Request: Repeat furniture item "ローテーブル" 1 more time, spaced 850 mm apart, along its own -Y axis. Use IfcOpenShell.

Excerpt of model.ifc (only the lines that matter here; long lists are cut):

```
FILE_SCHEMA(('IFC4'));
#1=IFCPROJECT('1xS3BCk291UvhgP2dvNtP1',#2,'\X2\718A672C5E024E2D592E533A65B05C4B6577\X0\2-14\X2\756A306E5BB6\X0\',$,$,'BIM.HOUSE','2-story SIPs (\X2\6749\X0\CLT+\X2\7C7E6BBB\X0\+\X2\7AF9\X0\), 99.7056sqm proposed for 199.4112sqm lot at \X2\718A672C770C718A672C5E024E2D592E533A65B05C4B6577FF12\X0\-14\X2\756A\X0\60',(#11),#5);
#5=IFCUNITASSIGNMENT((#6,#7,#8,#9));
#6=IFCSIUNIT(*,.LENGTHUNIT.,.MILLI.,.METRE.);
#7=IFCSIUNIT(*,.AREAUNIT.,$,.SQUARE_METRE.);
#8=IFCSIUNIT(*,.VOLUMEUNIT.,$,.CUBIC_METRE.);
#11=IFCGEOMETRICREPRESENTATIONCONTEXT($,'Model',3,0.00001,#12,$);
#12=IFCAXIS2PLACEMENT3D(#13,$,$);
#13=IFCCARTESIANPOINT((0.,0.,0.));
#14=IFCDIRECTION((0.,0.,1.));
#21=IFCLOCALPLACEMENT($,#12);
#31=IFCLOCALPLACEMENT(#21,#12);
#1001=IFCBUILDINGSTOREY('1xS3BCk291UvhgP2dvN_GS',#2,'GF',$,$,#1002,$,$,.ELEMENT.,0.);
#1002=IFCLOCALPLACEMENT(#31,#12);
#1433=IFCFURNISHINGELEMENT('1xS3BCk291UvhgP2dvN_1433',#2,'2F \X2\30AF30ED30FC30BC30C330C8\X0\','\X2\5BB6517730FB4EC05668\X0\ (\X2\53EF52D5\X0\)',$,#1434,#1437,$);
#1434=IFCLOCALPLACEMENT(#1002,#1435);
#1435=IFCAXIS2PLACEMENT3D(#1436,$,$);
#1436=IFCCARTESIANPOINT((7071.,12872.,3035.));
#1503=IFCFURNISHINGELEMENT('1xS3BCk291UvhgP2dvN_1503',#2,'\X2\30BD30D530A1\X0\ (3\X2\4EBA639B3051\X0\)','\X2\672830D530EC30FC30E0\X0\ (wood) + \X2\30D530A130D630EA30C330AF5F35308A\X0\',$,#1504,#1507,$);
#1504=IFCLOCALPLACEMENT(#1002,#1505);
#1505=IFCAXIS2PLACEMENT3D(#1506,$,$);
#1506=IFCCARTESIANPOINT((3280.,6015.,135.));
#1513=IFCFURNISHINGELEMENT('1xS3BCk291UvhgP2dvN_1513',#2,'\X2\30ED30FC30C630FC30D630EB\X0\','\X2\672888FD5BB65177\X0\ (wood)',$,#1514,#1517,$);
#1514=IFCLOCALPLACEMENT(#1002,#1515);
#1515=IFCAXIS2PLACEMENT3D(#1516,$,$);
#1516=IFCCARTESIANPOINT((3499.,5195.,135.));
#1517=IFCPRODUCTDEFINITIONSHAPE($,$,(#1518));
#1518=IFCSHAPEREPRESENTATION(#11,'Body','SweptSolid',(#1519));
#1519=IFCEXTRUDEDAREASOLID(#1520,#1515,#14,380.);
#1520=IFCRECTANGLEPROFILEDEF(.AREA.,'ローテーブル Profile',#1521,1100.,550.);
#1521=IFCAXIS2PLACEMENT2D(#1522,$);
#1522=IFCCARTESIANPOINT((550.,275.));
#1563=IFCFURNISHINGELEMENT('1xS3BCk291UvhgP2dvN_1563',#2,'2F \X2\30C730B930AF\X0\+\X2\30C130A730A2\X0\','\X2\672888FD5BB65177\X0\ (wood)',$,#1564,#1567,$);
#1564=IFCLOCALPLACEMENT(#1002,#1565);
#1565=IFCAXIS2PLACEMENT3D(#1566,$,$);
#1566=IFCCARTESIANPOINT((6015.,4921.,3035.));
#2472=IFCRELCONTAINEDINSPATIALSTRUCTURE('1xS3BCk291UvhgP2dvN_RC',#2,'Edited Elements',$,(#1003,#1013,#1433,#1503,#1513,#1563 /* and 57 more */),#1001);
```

```python
import ifcopenshell
import ifcopenshell.api.geometry
import ifcopenshell.api.root
import ifcopenshell.util.element
import ifcopenshell.util.placement

model = ifcopenshell.open("model.ifc")


def reuse_history(source, copy):
    """copy_class also copies each property set's owner history, people and application; keep the originals."""
    for rel in copy.IsDefinedBy:
        if rel.is_a("IfcRelDefinesByProperties") and (history := rel.RelatingPropertyDefinition.OwnerHistory):
            rel.RelatingPropertyDefinition.OwnerHistory = source.OwnerHistory
            ifcopenshell.util.element.remove_deep2(model, history)


source = model.by_guid("1xS3BCk291UvhgP2dvN_1513")
base = ifcopenshell.util.placement.get_local_placement(source.ObjectPlacement)
step = -base[:3, 1] * 850.0

for i in range(1, 2):
    copy = ifcopenshell.api.root.copy_class(model, product=source)
    copy.Representation = ifcopenshell.util.element.copy_deep(
        model, source.Representation, exclude=["IfcGeometricRepresentationContext", "IfcRepresentationMap"]
    )
    reuse_history(source, copy)
    matrix = base.copy()
    matrix[:3, 3] += i * step
    print("added at", matrix[:3, 3].round(3) + 0.0)
    ifcopenshell.api.geometry.edit_object_placement(model, product=copy, matrix=matrix, is_si=False)

model.write("model_v2.ifc")
```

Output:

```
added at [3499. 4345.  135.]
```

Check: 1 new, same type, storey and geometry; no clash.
